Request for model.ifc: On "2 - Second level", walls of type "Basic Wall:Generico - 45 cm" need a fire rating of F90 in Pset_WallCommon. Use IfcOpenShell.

First a look at what the model holds.

```python
import ifcopenshell
import ifcopenshell.util.element

model = ifcopenshell.open("model.ifc")
print(model.schema)
storey = next(s for s in model.by_type("IfcBuildingStorey") if s.Name == "2 - Second level")
walls = [e for e in ifcopenshell.util.element.get_decomposition(storey) if e.is_a("IfcWall")]
seen = {}
for e in walls:
    element_type = ifcopenshell.util.element.get_type(e)
    key = (element_type.Name if element_type != e and element_type else None, ifcopenshell.util.element.get_pset(e, "Pset_WallCommon", "FireRating"))
    seen[key] = seen.get(key, 0) + 1
for (name, value), count in sorted(seen.items(), key=str):
    print(count, "x", name, "|", value)
```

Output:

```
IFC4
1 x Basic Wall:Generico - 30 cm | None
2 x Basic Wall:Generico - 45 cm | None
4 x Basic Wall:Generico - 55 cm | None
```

```python
import ifcopenshell
import ifcopenshell.api.pset
import ifcopenshell.util.element

model = ifcopenshell.open("model.ifc")

storey = next(s for s in model.by_type("IfcBuildingStorey") if s.Name == "2 - Second level")
walls = [e for e in ifcopenshell.util.element.get_decomposition(storey) if e.is_a("IfcWall")]

count = 0
for e in walls:
    element_type = ifcopenshell.util.element.get_type(e)
    if element_type in (None, e) or element_type.Name != "Basic Wall:Generico - 45 cm":
        continue
    # add_pset returns the element's existing set when there is one.
    pset = ifcopenshell.api.pset.add_pset(model, product=e, name="Pset_WallCommon")
    ifcopenshell.api.pset.edit_pset(model, pset=pset, properties={"FireRating": "F90"})
    count += 1

print(count, "walls updated")

model.write("model_v2.ifc")
```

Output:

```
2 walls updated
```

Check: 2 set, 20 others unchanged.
